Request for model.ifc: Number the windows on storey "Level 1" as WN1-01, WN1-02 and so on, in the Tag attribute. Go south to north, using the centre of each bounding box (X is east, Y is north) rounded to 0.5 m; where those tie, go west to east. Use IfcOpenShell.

First a look at what the model holds.

```python
import ifcopenshell
import ifcopenshell.util.element
import ifcopenshell.util.placement

model = ifcopenshell.open("model.ifc")
print(model.schema)
storey = next(s for s in model.by_type("IfcBuildingStorey") if s.Name == "Level 1")
windows = [e for e in ifcopenshell.util.element.get_decomposition(storey) if e.is_a("IfcWindow")]
for e in sorted(windows, key=lambda e: e.id()):
    origin = ifcopenshell.util.placement.get_local_placement(e.ObjectPlacement)[:3, 3]
    print(e.id(), e.Tag, e.Name, origin.round(2) + 0.0, sep=" | ")
```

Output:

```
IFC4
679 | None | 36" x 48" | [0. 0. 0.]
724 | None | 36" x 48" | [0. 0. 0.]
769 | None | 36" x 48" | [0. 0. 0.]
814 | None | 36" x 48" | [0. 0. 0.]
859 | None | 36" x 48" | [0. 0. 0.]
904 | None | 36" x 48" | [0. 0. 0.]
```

```python
import ifcopenshell
import ifcopenshell.geom
import ifcopenshell.util.element
import ifcopenshell.util.shape

model = ifcopenshell.open("model.ifc")
settings = ifcopenshell.geom.settings()
settings.set("use-world-coords", True)


def centre(element):
    shape = ifcopenshell.geom.create_shape(settings, element)
    return ifcopenshell.util.shape.get_bbox_centroid(shape.geometry)


storey = next(s for s in model.by_type("IfcBuildingStorey") if s.Name == "Level 1")
windows = [e for e in ifcopenshell.util.element.get_decomposition(storey) if e.is_a("IfcWindow")]

# Insertion points can sit at a corner or the storey origin, so sort by the geometry (in metres).
centres = {e: centre(e) for e in windows}
windows.sort(key=lambda e: (round(centres[e][1] / 0.5), centres[e][0]))

for i, e in enumerate(windows, start=1):
    number = f"WN1-{i:02d}"
    e.Tag = number
    print(e.id(), number)

model.write("model_rev.ifc")
```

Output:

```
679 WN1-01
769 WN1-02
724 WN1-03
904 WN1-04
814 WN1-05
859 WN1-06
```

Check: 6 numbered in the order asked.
